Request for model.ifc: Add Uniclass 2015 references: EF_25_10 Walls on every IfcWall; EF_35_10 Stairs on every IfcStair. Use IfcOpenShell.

First a look at what the model holds.

```python
import ifcopenshell

model = ifcopenshell.open("model.ifc")
print(model.schema)
print("classifications:", [c.Name for c in model.by_type("IfcClassification")])
for ifc_class in ("IfcDoor", "IfcRoof", "IfcStair", "IfcWall", "IfcWindow"):
    print(ifc_class, len(model.by_type(ifc_class)))
```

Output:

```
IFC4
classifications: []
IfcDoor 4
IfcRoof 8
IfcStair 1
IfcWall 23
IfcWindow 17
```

```python
import ifcopenshell
import ifcopenshell.api.classification

model = ifcopenshell.open("model.ifc")

system = ifcopenshell.api.classification.add_classification(model, classification="Uniclass 2015")

codes = {
    "IfcWall": ("EF_25_10", "Walls"),
    "IfcStair": ("EF_35_10", "Stairs"),
}
for ifc_class, (code, name) in codes.items():
    products = model.by_type(ifc_class)
    ifcopenshell.api.classification.add_reference(
        model, products=products, classification=system, identification=code, name=name
    )
    print(code, len(products))

model.write("model_rev.ifc")
```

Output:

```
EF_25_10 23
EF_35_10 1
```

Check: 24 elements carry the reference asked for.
